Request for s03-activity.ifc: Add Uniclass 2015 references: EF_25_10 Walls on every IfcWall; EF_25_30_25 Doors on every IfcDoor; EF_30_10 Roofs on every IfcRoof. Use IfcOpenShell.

First a look at what the model holds.

```python
import ifcopenshell

model = ifcopenshell.open("s03-activity.ifc")
print(model.schema)
print("classifications:", [c.Name for c in model.by_type("IfcClassification")])
for ifc_class in ("IfcDoor", "IfcRoof", "IfcStair", "IfcWall", "IfcWindow"):
    print(ifc_class, len(model.by_type(ifc_class)))
```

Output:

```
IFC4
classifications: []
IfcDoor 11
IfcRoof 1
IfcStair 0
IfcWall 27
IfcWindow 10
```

```python
import ifcopenshell
import ifcopenshell.api.classification

model = ifcopenshell.open("s03-activity.ifc")

system = ifcopenshell.api.classification.add_classification(model, classification="Uniclass 2015")

codes = {
    "IfcWall": ("EF_25_10", "Walls"),
    "IfcDoor": ("EF_25_30_25", "Doors"),
    "IfcRoof": ("EF_30_10", "Roofs"),
}
for ifc_class, (code, name) in codes.items():
    products = model.by_type(ifc_class)
    ifcopenshell.api.classification.add_reference(
        model, products=products, classification=system, identification=code, name=name
    )
    print(code, len(products))

model.write("s03-activity_rev.ifc")
```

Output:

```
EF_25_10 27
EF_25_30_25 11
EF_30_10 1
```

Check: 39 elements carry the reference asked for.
